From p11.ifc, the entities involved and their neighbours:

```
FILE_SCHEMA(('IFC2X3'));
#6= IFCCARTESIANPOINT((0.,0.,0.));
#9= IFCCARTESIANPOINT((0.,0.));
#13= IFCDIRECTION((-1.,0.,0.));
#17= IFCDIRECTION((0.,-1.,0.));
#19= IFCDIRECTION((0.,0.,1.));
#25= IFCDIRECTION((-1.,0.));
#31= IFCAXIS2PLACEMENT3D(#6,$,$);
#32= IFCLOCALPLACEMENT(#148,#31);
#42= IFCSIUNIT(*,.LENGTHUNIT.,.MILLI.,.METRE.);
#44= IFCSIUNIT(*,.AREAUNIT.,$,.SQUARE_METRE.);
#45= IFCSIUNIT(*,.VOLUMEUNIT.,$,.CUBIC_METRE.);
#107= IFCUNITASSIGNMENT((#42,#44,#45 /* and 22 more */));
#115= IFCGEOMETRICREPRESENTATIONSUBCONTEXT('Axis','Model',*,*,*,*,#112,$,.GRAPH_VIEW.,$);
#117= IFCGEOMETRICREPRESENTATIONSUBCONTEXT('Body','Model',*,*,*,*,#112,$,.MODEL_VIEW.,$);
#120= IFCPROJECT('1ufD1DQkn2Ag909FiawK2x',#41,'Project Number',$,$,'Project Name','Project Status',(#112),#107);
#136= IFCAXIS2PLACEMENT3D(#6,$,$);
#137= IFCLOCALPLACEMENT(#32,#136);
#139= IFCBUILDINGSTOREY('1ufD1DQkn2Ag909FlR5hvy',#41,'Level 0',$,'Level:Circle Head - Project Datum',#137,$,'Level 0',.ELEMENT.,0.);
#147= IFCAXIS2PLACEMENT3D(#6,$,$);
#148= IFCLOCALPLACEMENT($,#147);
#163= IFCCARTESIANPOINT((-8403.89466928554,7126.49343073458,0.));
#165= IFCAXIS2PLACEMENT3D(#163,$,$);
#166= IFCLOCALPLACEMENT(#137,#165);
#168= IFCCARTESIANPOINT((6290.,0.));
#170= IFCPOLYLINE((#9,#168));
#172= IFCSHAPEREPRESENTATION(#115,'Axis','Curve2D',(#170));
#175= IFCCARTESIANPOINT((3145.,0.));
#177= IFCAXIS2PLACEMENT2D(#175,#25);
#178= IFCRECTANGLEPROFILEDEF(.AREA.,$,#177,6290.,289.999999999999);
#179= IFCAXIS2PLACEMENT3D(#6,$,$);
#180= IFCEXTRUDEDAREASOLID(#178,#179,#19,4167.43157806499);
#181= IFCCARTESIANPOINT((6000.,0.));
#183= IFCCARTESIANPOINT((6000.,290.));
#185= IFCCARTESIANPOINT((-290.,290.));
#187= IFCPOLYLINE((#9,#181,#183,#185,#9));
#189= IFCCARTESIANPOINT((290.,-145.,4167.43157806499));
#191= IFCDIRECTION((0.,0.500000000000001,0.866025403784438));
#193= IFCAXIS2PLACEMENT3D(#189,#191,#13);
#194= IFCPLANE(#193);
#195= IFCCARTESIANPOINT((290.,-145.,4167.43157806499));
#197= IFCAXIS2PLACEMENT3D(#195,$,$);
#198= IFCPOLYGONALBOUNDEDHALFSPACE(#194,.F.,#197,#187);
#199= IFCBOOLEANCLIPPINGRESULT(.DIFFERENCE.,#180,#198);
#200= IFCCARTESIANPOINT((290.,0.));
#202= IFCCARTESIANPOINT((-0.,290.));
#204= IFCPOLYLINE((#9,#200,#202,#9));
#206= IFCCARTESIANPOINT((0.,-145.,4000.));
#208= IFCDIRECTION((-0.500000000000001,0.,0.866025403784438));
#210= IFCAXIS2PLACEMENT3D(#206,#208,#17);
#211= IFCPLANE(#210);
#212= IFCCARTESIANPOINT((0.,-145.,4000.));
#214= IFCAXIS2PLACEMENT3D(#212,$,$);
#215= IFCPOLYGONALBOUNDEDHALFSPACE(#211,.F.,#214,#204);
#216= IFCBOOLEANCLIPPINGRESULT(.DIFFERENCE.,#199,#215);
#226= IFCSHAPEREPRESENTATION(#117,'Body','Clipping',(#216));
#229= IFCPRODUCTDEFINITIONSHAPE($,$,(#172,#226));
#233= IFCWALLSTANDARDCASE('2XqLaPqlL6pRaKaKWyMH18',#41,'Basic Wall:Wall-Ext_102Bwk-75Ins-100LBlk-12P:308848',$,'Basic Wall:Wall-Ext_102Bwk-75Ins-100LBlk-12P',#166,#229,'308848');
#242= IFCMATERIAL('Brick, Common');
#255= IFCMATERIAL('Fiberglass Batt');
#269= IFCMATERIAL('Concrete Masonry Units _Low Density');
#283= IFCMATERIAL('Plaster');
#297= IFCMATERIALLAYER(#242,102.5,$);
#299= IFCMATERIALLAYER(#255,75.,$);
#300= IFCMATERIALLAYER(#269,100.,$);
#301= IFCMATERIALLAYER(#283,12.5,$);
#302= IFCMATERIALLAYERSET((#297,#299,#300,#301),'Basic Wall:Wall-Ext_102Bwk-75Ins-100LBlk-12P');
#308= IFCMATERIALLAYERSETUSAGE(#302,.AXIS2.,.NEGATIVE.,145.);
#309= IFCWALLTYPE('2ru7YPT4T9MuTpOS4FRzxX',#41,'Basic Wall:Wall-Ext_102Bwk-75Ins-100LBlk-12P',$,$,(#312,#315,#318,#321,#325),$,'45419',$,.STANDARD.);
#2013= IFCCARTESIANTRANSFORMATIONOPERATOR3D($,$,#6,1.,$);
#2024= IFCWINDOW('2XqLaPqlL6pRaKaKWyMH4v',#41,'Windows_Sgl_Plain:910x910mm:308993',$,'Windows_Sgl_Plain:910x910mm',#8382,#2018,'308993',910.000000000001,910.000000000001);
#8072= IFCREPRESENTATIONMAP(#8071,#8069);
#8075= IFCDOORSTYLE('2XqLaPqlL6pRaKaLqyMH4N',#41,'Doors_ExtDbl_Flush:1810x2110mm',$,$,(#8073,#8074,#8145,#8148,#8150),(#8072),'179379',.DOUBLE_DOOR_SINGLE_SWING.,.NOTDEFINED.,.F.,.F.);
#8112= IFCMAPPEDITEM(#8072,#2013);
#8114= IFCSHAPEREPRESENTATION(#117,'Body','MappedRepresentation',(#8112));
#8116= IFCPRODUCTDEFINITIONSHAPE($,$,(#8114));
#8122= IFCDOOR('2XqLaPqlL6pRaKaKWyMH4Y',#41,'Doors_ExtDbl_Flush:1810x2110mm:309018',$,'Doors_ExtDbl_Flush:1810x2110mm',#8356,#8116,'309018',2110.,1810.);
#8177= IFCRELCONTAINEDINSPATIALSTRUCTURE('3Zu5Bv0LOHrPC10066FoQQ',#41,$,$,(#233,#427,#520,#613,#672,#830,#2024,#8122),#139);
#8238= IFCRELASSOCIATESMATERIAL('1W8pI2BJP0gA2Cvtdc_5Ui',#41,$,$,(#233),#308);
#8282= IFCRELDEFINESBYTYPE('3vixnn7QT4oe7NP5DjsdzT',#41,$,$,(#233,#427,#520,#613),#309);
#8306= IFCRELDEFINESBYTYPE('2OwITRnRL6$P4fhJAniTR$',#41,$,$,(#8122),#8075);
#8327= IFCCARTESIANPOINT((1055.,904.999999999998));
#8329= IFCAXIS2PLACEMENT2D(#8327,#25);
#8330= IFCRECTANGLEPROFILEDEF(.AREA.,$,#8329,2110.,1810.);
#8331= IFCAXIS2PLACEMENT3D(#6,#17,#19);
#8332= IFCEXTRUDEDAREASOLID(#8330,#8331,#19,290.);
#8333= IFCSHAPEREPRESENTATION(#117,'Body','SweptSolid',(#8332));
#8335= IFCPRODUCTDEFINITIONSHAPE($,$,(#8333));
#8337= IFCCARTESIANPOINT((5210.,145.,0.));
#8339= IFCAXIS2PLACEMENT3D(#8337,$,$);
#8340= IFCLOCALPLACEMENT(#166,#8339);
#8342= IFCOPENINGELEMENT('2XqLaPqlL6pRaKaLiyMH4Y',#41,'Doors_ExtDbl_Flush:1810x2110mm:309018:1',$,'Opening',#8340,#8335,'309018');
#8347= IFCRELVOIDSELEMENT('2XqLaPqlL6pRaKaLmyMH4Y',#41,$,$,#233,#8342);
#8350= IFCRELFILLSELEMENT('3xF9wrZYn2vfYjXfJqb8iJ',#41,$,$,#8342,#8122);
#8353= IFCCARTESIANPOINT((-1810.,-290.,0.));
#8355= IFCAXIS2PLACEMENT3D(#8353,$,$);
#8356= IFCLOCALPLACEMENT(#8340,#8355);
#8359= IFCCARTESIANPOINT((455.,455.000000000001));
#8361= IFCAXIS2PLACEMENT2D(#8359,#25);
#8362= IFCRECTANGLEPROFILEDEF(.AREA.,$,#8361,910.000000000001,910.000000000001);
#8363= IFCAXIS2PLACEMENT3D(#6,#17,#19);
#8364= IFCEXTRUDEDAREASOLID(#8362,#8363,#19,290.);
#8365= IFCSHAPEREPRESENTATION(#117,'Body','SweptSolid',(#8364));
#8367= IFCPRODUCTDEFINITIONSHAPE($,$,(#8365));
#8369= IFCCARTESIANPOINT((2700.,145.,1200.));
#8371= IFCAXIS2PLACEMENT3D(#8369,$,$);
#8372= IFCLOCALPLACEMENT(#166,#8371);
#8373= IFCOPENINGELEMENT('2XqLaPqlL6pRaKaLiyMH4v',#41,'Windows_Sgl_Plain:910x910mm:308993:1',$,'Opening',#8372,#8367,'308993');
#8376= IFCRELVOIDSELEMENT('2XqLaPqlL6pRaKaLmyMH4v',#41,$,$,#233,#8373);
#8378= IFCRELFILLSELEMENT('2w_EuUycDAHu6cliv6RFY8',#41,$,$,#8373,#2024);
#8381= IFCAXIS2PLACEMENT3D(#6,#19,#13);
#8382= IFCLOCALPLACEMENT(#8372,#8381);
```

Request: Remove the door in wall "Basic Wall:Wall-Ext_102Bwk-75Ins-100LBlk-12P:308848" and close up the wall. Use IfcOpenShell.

```python
import ifcopenshell
import ifcopenshell.api.feature
import ifcopenshell.api.root
import ifcopenshell.geom
import ifcopenshell.util.shape

model = ifcopenshell.open("p11.ifc")
settings = ifcopenshell.geom.settings()


def volume(element):
    """Net volume in cubic metres, openings subtracted."""
    shape = ifcopenshell.geom.create_shape(settings, element)
    return ifcopenshell.util.shape.get_volume(shape.geometry)


door = model.by_guid("2XqLaPqlL6pRaKaKWyMH4Y")
opening = door.FillsVoids[0].RelatingOpeningElement
wall = opening.VoidsElements[0].RelatingBuildingElement
before = volume(wall)

ifcopenshell.api.root.remove_product(model, product=door)
ifcopenshell.api.feature.remove_feature(model, feature=opening)

after = volume(wall)

print(f"wall volume {before:.3f} -> {after:.3f} m3")

model.write("p11_rev.ifc")
```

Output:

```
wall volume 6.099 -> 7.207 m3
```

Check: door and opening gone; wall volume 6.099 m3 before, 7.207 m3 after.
